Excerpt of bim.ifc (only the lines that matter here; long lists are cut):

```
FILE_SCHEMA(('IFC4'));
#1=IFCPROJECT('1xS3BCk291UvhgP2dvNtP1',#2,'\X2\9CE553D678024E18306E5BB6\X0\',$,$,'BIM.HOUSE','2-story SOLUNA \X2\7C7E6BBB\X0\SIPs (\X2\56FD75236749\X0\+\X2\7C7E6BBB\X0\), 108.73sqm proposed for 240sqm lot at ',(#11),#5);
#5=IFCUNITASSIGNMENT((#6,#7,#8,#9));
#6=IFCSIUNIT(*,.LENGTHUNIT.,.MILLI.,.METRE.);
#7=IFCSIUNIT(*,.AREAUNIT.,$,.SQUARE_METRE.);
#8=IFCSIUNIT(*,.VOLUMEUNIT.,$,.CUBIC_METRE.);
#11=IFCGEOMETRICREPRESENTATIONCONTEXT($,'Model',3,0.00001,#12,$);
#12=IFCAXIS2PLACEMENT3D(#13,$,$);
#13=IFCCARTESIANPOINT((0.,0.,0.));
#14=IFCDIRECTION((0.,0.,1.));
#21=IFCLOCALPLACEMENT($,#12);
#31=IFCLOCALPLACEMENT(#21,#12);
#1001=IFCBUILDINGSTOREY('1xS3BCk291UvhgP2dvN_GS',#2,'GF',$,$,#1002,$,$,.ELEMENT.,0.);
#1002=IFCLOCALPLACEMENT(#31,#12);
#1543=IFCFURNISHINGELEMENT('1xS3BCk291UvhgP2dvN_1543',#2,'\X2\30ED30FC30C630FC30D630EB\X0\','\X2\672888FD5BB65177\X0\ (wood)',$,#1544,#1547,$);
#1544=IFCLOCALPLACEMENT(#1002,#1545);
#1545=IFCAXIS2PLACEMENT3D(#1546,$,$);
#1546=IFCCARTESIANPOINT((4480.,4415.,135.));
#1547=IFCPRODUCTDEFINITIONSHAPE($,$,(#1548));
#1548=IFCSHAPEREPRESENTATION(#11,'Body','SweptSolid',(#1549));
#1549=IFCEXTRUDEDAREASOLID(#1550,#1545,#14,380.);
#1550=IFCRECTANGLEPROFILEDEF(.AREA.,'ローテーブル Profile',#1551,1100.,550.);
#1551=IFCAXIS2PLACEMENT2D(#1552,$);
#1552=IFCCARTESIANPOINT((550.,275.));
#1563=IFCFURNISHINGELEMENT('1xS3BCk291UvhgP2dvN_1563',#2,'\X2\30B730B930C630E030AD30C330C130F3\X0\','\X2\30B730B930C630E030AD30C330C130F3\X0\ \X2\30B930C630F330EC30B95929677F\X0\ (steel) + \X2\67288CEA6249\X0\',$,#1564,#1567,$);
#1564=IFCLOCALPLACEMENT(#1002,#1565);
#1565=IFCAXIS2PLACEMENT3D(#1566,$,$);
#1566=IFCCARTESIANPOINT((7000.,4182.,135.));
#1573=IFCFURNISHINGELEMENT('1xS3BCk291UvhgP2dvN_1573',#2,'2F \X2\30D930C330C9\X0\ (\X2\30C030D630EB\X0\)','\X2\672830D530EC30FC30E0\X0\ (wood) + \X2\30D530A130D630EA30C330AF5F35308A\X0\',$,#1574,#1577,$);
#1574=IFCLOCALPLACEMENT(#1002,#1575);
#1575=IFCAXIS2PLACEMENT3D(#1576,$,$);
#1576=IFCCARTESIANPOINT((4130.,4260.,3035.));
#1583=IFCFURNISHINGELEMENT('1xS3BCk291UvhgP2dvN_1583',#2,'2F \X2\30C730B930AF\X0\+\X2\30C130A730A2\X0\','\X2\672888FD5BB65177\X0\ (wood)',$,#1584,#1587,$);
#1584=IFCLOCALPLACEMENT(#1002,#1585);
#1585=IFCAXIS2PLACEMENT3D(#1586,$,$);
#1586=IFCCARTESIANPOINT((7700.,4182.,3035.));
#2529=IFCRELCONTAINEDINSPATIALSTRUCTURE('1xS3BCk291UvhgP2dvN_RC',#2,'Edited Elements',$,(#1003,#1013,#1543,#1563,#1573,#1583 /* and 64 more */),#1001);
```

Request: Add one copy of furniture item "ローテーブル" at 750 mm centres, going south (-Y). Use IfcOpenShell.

```python
import numpy as np
import ifcopenshell
import ifcopenshell.api.geometry
import ifcopenshell.api.root
import ifcopenshell.util.element
import ifcopenshell.util.placement

model = ifcopenshell.open("bim.ifc")


def reuse_history(source, copy):
    """copy_class also copies each property set's owner history, people and application; keep the originals."""
    for rel in copy.IsDefinedBy:
        if rel.is_a("IfcRelDefinesByProperties") and (history := rel.RelatingPropertyDefinition.OwnerHistory):
            rel.RelatingPropertyDefinition.OwnerHistory = source.OwnerHistory
            ifcopenshell.util.element.remove_deep2(model, history)


source = model.by_guid("1xS3BCk291UvhgP2dvN_1543")
base = ifcopenshell.util.placement.get_local_placement(source.ObjectPlacement)
step = np.array([0.0, -1.0, 0.0]) * 750.0

for i in range(1, 2):
    copy = ifcopenshell.api.root.copy_class(model, product=source)
    copy.Representation = ifcopenshell.util.element.copy_deep(
        model, source.Representation, exclude=["IfcGeometricRepresentationContext", "IfcRepresentationMap"]
    )
    reuse_history(source, copy)
    matrix = base.copy()
    matrix[:3, 3] += i * step
    print("added at", matrix[:3, 3].round(3) + 0.0)
    ifcopenshell.api.geometry.edit_object_placement(model, product=copy, matrix=matrix, is_si=False)

model.write("bim_rev.ifc")
```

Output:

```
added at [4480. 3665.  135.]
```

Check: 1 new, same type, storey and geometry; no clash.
